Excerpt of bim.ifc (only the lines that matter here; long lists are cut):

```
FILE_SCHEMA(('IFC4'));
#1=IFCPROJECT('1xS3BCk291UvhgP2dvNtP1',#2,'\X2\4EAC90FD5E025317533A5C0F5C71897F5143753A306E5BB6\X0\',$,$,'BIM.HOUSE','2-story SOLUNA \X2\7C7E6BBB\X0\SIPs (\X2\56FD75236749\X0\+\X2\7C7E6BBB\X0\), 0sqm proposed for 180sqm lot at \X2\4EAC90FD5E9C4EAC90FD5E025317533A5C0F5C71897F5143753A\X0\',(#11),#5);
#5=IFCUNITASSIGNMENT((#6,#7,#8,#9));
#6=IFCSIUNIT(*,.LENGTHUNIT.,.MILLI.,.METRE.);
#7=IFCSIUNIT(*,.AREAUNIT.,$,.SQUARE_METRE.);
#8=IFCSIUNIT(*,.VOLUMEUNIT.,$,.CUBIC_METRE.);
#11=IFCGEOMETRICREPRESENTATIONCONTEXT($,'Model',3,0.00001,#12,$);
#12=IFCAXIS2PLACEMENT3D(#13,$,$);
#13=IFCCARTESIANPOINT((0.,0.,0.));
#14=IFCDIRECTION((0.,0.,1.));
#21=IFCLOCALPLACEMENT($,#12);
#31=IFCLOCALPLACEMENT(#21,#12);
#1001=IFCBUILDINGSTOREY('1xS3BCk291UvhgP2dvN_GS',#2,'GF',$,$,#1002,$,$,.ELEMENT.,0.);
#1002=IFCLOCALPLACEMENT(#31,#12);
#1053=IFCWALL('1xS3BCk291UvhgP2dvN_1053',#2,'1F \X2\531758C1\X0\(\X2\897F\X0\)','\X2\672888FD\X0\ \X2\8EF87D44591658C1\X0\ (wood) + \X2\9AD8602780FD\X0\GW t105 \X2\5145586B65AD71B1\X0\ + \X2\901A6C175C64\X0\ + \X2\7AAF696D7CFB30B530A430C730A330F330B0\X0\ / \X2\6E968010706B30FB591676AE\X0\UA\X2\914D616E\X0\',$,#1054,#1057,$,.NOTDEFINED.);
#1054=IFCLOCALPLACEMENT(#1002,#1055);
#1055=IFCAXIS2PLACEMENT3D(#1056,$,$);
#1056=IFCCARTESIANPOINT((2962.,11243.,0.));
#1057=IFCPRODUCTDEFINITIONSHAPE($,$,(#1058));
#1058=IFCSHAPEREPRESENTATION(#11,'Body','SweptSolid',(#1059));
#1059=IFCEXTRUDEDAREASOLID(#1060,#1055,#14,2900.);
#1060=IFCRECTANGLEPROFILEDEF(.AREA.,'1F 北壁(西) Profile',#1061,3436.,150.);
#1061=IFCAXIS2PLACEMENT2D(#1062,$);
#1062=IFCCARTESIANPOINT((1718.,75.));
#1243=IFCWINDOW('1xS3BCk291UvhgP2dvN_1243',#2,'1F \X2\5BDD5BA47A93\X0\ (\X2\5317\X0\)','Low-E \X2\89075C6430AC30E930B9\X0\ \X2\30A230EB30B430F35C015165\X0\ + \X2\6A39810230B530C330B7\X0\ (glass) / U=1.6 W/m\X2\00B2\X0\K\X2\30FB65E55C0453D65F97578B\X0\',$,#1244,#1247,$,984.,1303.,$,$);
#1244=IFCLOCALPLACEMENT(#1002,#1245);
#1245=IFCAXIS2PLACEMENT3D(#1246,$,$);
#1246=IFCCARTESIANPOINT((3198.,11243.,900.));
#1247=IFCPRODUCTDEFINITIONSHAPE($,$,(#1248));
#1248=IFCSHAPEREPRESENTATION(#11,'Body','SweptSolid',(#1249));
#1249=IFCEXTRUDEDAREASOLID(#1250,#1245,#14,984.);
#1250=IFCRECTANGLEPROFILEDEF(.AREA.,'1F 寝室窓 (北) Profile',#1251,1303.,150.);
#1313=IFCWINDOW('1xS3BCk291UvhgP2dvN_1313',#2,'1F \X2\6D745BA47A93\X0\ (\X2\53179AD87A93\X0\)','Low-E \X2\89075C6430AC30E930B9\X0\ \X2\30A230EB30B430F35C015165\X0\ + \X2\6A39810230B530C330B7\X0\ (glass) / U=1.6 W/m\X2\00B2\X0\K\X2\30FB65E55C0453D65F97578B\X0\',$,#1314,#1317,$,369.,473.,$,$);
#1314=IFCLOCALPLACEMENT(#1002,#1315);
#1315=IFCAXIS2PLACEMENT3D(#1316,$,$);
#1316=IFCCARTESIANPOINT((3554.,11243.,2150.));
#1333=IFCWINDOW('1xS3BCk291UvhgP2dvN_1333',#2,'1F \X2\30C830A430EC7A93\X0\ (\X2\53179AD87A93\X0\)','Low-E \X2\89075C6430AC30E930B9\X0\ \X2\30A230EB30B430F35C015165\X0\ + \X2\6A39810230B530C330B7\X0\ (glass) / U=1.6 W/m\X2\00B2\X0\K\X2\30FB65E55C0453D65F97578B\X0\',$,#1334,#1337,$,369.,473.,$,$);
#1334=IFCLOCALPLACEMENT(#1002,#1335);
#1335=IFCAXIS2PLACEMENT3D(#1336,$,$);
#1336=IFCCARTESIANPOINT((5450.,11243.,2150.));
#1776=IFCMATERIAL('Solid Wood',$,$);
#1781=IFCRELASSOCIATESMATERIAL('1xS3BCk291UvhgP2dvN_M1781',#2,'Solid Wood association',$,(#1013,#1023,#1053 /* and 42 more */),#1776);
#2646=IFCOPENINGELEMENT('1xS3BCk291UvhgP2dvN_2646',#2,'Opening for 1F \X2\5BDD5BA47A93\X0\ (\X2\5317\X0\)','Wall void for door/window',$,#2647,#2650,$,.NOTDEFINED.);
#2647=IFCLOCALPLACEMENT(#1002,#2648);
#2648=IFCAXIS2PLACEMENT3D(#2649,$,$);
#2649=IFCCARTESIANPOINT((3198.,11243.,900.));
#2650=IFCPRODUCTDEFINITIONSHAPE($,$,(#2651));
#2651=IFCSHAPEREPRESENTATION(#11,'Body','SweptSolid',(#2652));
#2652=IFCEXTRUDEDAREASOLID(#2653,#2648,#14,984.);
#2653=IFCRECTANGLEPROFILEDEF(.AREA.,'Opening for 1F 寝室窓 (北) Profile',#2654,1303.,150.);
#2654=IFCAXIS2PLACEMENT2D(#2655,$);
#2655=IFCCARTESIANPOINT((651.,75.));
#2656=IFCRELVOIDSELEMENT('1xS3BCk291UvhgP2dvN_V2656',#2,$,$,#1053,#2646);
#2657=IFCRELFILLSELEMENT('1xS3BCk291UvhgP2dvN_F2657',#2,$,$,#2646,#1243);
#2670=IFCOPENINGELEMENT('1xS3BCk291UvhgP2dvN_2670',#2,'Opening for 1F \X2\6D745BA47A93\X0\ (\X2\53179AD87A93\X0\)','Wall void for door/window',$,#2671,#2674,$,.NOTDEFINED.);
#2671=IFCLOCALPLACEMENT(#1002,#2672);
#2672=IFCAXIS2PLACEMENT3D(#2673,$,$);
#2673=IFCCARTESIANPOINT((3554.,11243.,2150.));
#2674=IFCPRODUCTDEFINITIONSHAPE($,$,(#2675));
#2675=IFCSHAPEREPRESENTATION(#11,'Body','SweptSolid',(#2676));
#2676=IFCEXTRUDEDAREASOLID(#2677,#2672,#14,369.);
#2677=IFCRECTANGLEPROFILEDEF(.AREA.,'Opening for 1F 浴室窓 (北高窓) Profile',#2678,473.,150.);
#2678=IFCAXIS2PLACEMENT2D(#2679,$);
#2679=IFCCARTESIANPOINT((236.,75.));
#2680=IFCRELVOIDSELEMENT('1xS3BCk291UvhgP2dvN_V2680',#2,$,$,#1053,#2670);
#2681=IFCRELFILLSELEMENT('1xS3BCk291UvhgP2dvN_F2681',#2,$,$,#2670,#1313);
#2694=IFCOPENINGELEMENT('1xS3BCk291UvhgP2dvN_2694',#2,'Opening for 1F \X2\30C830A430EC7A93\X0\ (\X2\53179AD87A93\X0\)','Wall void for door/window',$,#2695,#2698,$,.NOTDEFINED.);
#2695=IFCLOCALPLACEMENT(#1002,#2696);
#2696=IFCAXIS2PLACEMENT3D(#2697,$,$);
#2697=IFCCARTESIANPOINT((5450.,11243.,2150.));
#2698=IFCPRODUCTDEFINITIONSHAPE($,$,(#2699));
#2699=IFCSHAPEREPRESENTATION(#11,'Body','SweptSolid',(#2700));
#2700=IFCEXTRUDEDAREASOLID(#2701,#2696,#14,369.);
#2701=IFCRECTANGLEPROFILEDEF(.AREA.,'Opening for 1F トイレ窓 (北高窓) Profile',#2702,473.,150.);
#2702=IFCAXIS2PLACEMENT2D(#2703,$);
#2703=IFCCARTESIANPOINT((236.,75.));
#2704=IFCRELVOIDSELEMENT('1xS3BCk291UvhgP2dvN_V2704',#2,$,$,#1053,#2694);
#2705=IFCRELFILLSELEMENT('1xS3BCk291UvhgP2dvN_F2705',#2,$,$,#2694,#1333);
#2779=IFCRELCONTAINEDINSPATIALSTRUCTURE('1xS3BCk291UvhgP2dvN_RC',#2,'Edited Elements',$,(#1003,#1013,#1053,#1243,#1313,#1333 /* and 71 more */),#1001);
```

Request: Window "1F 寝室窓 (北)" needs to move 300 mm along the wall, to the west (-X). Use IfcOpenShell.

```python
import ifcopenshell
import ifcopenshell.api.geometry
import ifcopenshell.util.placement
import ifcopenshell.util.unit

model = ifcopenshell.open("bim.ifc")
unit_scale = ifcopenshell.util.unit.calculate_unit_scale(model)

window = model.by_guid("1xS3BCk291UvhgP2dvN_1243")
opening = window.FillsVoids[0].RelatingOpeningElement
wall = opening.VoidsElements[0].RelatingBuildingElement

wall_matrix = ifcopenshell.util.placement.get_local_placement(wall.ObjectPlacement)
shift = wall_matrix[:3, 0] * -0.3 / unit_scale
before = ifcopenshell.util.placement.get_local_placement(window.ObjectPlacement)[:3, 3].copy()

# The window is not placed relative to its opening, so move both.
for product in (opening, window):
    matrix = ifcopenshell.util.placement.get_local_placement(product.ObjectPlacement)
    matrix[:3, 3] += shift
    ifcopenshell.api.geometry.edit_object_placement(model, product=product, matrix=matrix, is_si=False)

after = ifcopenshell.util.placement.get_local_placement(window.ObjectPlacement)[:3, 3]
print("window moved by", (after - before).round(3) + 0.0)

model.write("bim_edited.ifc")
```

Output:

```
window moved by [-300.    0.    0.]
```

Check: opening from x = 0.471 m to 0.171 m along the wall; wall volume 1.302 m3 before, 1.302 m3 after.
